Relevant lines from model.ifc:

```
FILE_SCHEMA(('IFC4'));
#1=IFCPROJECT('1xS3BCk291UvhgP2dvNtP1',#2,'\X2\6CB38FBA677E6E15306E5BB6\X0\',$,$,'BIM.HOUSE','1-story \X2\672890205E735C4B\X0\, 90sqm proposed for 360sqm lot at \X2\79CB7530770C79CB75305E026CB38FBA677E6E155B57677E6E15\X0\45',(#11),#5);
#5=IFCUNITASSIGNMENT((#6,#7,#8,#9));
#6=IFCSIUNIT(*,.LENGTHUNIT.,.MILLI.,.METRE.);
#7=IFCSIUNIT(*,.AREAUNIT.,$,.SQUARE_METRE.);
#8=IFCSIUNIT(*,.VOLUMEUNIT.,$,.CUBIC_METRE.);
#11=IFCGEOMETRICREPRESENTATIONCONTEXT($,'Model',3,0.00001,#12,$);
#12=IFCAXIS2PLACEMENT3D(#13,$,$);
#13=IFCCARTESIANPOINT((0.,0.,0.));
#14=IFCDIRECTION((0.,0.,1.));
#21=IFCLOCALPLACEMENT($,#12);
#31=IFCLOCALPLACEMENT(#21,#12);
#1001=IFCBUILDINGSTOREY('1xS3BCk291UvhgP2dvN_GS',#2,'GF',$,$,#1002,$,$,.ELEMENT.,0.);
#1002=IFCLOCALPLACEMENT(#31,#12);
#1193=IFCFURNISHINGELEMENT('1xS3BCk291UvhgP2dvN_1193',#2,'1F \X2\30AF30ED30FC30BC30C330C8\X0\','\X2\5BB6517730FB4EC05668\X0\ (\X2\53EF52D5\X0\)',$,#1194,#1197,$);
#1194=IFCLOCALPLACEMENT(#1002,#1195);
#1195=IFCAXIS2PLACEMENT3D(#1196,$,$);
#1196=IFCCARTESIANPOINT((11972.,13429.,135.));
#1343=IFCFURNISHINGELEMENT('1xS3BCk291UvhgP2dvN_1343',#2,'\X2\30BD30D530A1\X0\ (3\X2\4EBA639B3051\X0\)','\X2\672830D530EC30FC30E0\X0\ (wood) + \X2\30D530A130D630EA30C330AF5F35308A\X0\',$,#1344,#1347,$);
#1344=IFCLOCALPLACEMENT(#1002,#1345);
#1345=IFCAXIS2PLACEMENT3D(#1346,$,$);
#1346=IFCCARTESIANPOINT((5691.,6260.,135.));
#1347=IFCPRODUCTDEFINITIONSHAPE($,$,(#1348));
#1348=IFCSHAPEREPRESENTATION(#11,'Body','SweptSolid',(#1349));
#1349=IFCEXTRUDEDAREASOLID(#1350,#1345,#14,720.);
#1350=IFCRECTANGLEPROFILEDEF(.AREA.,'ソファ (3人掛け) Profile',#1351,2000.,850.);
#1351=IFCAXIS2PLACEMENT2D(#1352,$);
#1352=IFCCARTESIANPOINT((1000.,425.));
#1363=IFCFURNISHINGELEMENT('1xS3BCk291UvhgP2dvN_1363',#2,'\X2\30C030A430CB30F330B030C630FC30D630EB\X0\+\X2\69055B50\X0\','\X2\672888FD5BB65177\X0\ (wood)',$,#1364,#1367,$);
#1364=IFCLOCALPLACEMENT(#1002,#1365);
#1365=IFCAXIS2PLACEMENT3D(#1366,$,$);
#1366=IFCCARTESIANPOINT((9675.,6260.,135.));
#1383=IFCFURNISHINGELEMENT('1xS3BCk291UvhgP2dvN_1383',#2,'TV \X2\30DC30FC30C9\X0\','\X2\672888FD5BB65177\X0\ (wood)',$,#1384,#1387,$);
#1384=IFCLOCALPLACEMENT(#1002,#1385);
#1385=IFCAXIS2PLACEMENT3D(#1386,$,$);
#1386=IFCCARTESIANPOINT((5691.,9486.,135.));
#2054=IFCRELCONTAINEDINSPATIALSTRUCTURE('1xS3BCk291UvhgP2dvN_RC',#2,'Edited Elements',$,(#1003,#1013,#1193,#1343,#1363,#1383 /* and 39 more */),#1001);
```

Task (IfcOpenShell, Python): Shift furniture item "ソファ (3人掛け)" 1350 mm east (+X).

```python
import ifcopenshell
import ifcopenshell.api.geometry
import ifcopenshell.util.placement
import ifcopenshell.util.unit

model = ifcopenshell.open("model.ifc")
unit_scale = ifcopenshell.util.unit.calculate_unit_scale(model)

item = model.by_guid("1xS3BCk291UvhgP2dvN_1343")
matrix = ifcopenshell.util.placement.get_local_placement(item.ObjectPlacement)
matrix[0, 3] += 1.35 / unit_scale
ifcopenshell.api.geometry.edit_object_placement(model, product=item, matrix=matrix, is_si=False)

print(ifcopenshell.util.placement.get_local_placement(item.ObjectPlacement).round(3) + 0.0)

model.write("model-out.ifc")
```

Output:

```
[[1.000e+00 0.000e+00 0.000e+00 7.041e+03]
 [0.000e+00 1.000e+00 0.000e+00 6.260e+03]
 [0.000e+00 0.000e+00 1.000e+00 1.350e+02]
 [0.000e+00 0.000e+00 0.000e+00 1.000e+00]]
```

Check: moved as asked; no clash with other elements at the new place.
